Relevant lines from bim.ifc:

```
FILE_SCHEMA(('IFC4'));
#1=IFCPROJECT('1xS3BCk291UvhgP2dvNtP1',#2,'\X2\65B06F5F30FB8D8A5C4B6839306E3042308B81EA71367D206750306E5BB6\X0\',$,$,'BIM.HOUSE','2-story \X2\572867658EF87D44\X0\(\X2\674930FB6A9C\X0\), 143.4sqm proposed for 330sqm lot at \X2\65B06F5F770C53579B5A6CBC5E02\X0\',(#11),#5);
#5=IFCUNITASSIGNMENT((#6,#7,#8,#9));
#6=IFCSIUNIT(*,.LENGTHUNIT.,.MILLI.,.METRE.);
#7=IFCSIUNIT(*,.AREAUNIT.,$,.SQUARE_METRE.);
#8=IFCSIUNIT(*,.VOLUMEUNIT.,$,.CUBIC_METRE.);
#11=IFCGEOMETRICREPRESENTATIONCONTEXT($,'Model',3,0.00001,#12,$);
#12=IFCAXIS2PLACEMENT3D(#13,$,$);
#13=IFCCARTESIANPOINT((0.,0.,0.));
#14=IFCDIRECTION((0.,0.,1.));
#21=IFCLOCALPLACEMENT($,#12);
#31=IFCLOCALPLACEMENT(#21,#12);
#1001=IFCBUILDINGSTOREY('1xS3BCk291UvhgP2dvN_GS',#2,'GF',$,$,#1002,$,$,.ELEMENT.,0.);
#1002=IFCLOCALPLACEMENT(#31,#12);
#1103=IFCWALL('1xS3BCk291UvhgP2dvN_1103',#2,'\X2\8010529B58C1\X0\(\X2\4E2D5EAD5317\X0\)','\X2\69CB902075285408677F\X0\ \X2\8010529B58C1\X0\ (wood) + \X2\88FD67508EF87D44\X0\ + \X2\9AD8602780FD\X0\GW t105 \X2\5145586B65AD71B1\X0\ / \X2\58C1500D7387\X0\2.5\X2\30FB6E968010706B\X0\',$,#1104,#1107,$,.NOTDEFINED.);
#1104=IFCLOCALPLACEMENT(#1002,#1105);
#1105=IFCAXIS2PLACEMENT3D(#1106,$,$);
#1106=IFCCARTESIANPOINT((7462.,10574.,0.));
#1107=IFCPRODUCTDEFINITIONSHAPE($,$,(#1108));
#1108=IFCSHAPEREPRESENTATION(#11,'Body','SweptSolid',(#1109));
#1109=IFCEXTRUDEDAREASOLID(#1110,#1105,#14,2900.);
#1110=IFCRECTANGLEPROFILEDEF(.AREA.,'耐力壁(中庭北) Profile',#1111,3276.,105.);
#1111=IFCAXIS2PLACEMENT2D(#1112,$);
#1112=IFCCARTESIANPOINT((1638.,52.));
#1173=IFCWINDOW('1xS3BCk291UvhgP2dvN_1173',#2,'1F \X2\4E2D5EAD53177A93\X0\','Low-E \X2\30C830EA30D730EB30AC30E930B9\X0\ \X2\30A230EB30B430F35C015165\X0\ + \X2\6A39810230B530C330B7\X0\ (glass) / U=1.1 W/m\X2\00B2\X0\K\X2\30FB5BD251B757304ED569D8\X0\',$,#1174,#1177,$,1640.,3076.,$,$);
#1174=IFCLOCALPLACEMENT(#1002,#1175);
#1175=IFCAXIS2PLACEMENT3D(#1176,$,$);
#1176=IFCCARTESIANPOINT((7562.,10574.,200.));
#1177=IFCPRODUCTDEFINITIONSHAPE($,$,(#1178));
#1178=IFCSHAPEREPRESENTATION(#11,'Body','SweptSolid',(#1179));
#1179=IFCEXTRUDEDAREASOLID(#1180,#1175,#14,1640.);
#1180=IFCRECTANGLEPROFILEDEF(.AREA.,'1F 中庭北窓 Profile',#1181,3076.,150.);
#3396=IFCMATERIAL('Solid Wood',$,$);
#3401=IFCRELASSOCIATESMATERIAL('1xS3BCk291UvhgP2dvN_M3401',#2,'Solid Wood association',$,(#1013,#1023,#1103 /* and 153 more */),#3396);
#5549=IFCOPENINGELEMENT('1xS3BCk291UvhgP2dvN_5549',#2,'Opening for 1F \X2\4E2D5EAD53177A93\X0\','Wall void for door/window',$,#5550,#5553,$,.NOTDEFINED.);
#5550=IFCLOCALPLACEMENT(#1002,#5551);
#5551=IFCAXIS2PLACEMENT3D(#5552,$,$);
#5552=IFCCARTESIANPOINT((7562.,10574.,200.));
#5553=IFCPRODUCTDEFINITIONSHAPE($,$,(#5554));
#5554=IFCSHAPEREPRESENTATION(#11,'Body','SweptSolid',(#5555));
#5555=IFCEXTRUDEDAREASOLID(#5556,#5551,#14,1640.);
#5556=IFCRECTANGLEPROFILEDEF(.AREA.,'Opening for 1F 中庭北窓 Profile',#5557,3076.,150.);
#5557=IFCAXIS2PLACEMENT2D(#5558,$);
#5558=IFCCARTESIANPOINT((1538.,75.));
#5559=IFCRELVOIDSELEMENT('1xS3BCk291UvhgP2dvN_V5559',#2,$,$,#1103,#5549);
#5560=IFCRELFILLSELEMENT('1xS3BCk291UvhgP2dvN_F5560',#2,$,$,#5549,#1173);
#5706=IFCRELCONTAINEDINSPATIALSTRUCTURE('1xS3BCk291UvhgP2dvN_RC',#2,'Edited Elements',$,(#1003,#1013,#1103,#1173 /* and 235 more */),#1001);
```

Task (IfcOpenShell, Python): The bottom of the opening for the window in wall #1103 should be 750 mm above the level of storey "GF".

```python
import numpy as np
import ifcopenshell
import ifcopenshell.api.geometry
import ifcopenshell.geom
import ifcopenshell.util.element
import ifcopenshell.util.placement
import ifcopenshell.util.shape
import ifcopenshell.util.unit

model = ifcopenshell.open("bim.ifc")
unit_scale = ifcopenshell.util.unit.calculate_unit_scale(model)

window = model.by_guid("1xS3BCk291UvhgP2dvN_1173")
opening = window.FillsVoids[0].RelatingOpeningElement
storey = ifcopenshell.util.element.get_container(window, ifc_class="IfcBuildingStorey")
level = ifcopenshell.util.placement.get_local_placement(storey.ObjectPlacement)[2, 3]

# The opening's origin need not be at the sill, so measure its lowest point.
shape = ifcopenshell.geom.create_shape(ifcopenshell.geom.settings(), opening)
bottom = ifcopenshell.util.shape.get_shape_bottom_elevation(shape, shape.geometry) / unit_scale
dz = level + 750.0 - bottom

shift = np.array([0.0, 0.0, dz])
# The window is not placed relative to its opening, so move both.
for product in (opening, window):
    matrix = ifcopenshell.util.placement.get_local_placement(product.ObjectPlacement)
    matrix[:3, 3] += shift
    ifcopenshell.api.geometry.edit_object_placement(model, product=product, matrix=matrix, is_si=False)

print(f"moved by {dz * unit_scale:+.3f} m")

model.write("bim_rev.ifc")
```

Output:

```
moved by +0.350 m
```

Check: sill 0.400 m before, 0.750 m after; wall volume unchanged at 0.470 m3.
